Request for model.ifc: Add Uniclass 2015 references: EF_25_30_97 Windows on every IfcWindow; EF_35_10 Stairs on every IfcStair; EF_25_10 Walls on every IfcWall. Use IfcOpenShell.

First a look at what the model holds.

```python
import ifcopenshell

model = ifcopenshell.open("model.ifc")
print(model.schema)
print("classifications:", [c.Name for c in model.by_type("IfcClassification")])
for ifc_class in ("IfcDoor", "IfcRoof", "IfcStair", "IfcWall", "IfcWindow"):
    print(ifc_class, len(model.by_type(ifc_class)))
```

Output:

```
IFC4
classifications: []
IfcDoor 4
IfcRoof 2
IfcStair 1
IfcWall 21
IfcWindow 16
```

```python
import ifcopenshell
import ifcopenshell.api.classification

model = ifcopenshell.open("model.ifc")

system = ifcopenshell.api.classification.add_classification(model, classification="Uniclass 2015")

codes = {
    "IfcWindow": ("EF_25_30_97", "Windows"),
    "IfcStair": ("EF_35_10", "Stairs"),
    "IfcWall": ("EF_25_10", "Walls"),
}
for ifc_class, (code, name) in codes.items():
    products = model.by_type(ifc_class)
    ifcopenshell.api.classification.add_reference(
        model, products=products, classification=system, identification=code, name=name
    )
    print(code, len(products))

model.write("model_updated.ifc")
```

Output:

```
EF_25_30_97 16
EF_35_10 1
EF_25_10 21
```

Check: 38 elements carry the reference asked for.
